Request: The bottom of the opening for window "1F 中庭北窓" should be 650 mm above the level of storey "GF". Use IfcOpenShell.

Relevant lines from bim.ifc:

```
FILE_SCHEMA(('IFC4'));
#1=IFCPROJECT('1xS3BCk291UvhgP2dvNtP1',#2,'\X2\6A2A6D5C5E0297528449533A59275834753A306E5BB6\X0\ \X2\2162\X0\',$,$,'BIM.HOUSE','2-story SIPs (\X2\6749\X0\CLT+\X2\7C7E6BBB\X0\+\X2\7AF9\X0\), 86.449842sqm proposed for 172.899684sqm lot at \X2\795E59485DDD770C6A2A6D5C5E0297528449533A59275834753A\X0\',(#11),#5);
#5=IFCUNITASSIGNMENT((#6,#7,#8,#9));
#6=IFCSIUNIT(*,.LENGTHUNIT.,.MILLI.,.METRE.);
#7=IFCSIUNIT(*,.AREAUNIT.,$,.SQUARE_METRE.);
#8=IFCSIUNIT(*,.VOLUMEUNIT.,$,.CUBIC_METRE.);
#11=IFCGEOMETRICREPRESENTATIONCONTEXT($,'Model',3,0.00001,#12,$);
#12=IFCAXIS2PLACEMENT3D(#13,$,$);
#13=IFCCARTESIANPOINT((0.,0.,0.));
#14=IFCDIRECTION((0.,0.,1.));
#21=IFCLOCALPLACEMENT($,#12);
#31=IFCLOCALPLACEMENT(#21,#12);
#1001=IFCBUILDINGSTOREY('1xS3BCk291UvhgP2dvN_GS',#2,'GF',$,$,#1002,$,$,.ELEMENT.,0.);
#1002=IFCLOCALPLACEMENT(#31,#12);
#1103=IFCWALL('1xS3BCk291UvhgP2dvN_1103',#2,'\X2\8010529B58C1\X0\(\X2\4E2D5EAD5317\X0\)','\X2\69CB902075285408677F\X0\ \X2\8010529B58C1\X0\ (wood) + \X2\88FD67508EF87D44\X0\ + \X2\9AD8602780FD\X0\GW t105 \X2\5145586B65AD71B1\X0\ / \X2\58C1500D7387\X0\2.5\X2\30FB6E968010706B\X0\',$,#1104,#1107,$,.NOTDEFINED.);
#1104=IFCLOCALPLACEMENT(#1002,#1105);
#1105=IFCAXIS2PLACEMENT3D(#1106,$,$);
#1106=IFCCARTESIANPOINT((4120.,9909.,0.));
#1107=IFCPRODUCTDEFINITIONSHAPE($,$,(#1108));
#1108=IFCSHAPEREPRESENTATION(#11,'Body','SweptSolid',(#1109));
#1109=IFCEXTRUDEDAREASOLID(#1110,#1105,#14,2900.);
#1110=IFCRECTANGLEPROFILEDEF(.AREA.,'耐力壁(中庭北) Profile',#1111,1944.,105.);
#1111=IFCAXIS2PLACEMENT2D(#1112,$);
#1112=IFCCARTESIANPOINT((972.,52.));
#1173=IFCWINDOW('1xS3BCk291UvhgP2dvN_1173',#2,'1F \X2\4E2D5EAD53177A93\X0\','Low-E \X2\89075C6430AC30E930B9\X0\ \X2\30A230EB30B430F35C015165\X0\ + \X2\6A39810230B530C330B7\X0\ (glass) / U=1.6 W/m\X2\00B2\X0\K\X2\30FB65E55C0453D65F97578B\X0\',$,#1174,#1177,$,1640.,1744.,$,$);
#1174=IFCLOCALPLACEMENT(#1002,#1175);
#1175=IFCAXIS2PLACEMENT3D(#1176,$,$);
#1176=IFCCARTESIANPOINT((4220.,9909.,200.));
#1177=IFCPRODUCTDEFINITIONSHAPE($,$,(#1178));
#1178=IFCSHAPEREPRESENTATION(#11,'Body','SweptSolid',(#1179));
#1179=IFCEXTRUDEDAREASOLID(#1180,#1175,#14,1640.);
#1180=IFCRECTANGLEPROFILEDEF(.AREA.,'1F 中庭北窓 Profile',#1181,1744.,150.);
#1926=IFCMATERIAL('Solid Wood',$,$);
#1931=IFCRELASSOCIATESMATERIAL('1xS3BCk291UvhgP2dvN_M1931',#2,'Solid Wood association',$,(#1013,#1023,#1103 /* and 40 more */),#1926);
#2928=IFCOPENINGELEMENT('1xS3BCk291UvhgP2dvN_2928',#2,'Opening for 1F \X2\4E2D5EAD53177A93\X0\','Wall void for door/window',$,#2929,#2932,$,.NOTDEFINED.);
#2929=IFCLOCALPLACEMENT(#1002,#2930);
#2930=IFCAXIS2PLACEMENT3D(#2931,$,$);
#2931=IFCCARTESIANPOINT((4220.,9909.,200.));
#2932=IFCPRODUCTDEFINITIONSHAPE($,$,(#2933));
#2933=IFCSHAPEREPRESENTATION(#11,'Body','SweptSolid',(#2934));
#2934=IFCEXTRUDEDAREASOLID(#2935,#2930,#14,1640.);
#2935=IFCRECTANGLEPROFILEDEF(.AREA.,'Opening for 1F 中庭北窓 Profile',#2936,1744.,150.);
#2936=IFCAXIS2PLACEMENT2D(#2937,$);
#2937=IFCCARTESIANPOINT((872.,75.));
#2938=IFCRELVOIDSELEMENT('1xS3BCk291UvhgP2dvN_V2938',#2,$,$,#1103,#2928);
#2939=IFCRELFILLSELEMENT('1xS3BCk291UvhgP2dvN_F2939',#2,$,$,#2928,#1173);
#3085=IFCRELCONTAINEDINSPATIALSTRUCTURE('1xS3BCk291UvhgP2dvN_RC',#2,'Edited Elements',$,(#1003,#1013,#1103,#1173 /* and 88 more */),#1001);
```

```python
import numpy as np
import ifcopenshell
import ifcopenshell.api.geometry
import ifcopenshell.geom
import ifcopenshell.util.element
import ifcopenshell.util.placement
import ifcopenshell.util.shape
import ifcopenshell.util.unit

model = ifcopenshell.open("bim.ifc")
unit_scale = ifcopenshell.util.unit.calculate_unit_scale(model)

window = model.by_guid("1xS3BCk291UvhgP2dvN_1173")
opening = window.FillsVoids[0].RelatingOpeningElement
storey = ifcopenshell.util.element.get_container(window, ifc_class="IfcBuildingStorey")
level = ifcopenshell.util.placement.get_local_placement(storey.ObjectPlacement)[2, 3]

# The opening's origin need not be at the sill, so measure its lowest point.
shape = ifcopenshell.geom.create_shape(ifcopenshell.geom.settings(), opening)
bottom = ifcopenshell.util.shape.get_shape_bottom_elevation(shape, shape.geometry) / unit_scale
dz = level + 0.65 / unit_scale - bottom

shift = np.array([0.0, 0.0, dz])
# The window is not placed relative to its opening, so move both.
for product in (opening, window):
    matrix = ifcopenshell.util.placement.get_local_placement(product.ObjectPlacement)
    matrix[:3, 3] += shift
    ifcopenshell.api.geometry.edit_object_placement(model, product=product, matrix=matrix, is_si=False)

print(f"moved by {dz * unit_scale:+.3f} m")

model.write("bim_edited.ifc")
```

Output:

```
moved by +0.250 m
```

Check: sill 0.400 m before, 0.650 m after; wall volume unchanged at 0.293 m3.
